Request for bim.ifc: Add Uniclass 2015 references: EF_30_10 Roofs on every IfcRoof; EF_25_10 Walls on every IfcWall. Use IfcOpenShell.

First a look at what the model holds.

```python
import ifcopenshell

model = ifcopenshell.open("bim.ifc")
print(model.schema)
print("classifications:", [c.Name for c in model.by_type("IfcClassification")])
for ifc_class in ("IfcDoor", "IfcRoof", "IfcStair", "IfcWall", "IfcWindow"):
    print(ifc_class, len(model.by_type(ifc_class)))
```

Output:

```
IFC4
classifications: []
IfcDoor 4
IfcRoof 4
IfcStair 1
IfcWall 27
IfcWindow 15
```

```python
import ifcopenshell
import ifcopenshell.api.classification

model = ifcopenshell.open("bim.ifc")

system = ifcopenshell.api.classification.add_classification(model, classification="Uniclass 2015")

codes = {
    "IfcRoof": ("EF_30_10", "Roofs"),
    "IfcWall": ("EF_25_10", "Walls"),
}
for ifc_class, (code, name) in codes.items():
    products = model.by_type(ifc_class)
    ifcopenshell.api.classification.add_reference(
        model, products=products, classification=system, identification=code, name=name
    )
    print(code, len(products))

model.write("bim_edited.ifc")
```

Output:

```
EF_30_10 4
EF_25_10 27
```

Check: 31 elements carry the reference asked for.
